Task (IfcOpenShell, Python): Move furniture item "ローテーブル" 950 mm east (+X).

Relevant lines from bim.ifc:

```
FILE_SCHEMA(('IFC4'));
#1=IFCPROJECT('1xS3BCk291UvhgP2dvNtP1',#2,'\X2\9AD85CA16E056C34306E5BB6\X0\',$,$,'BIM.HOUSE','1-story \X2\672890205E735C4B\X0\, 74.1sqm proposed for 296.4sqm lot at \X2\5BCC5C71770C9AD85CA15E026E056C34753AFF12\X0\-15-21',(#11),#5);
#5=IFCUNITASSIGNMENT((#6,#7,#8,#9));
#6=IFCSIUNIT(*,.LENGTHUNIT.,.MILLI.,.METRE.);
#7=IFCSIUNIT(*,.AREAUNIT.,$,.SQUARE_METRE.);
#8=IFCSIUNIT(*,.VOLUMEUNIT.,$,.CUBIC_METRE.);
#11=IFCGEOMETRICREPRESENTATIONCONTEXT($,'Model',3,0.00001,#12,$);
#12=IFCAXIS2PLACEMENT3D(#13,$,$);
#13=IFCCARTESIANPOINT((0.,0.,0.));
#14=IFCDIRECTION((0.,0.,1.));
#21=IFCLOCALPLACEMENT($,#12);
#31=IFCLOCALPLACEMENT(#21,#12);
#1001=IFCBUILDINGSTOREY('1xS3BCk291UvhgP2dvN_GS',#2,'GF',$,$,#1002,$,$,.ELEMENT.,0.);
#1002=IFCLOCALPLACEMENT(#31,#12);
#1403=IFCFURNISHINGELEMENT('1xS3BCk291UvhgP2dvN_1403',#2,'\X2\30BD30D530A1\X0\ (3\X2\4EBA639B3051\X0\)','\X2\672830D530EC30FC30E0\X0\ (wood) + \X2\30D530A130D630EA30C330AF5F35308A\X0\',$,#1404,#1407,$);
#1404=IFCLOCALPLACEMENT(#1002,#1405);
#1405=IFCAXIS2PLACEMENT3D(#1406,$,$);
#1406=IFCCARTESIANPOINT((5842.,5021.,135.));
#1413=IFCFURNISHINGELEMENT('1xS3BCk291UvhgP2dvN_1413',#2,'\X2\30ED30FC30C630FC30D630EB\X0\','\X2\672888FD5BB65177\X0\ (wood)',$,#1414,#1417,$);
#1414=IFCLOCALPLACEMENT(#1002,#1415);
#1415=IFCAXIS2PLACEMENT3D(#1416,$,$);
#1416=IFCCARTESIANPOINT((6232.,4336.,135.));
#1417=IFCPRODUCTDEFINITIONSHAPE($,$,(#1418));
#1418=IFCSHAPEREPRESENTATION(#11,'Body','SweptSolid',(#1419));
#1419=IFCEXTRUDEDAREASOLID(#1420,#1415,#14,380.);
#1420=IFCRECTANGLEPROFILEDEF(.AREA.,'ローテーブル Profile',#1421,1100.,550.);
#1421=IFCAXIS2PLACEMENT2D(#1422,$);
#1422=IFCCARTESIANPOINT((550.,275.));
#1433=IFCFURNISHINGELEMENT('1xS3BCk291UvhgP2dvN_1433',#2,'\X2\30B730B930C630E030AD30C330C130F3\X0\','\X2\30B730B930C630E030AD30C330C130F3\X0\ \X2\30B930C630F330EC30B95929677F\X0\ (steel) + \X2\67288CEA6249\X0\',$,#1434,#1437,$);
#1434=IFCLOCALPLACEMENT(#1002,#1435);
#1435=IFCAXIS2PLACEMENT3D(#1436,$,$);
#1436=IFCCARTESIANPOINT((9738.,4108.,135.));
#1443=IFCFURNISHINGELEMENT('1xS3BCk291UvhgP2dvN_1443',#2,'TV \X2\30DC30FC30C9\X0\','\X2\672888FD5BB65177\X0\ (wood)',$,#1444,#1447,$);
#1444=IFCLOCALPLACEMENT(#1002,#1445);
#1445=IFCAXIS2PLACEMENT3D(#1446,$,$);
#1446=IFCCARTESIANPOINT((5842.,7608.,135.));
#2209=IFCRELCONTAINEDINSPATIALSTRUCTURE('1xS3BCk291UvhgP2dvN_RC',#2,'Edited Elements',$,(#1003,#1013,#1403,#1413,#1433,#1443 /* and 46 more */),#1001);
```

```python
import ifcopenshell
import ifcopenshell.api.geometry
import ifcopenshell.util.placement
import ifcopenshell.util.unit

model = ifcopenshell.open("bim.ifc")
unit_scale = ifcopenshell.util.unit.calculate_unit_scale(model)

item = model.by_guid("1xS3BCk291UvhgP2dvN_1413")
matrix = ifcopenshell.util.placement.get_local_placement(item.ObjectPlacement)
matrix[0, 3] += 0.95 / unit_scale
ifcopenshell.api.geometry.edit_object_placement(model, product=item, matrix=matrix, is_si=False)

print(ifcopenshell.util.placement.get_local_placement(item.ObjectPlacement).round(3) + 0.0)

model.write("bim_v2.ifc")
```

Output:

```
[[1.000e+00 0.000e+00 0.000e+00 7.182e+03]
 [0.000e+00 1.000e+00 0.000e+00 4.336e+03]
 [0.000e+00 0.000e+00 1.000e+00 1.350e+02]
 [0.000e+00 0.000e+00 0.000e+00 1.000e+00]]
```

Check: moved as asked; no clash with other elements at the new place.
